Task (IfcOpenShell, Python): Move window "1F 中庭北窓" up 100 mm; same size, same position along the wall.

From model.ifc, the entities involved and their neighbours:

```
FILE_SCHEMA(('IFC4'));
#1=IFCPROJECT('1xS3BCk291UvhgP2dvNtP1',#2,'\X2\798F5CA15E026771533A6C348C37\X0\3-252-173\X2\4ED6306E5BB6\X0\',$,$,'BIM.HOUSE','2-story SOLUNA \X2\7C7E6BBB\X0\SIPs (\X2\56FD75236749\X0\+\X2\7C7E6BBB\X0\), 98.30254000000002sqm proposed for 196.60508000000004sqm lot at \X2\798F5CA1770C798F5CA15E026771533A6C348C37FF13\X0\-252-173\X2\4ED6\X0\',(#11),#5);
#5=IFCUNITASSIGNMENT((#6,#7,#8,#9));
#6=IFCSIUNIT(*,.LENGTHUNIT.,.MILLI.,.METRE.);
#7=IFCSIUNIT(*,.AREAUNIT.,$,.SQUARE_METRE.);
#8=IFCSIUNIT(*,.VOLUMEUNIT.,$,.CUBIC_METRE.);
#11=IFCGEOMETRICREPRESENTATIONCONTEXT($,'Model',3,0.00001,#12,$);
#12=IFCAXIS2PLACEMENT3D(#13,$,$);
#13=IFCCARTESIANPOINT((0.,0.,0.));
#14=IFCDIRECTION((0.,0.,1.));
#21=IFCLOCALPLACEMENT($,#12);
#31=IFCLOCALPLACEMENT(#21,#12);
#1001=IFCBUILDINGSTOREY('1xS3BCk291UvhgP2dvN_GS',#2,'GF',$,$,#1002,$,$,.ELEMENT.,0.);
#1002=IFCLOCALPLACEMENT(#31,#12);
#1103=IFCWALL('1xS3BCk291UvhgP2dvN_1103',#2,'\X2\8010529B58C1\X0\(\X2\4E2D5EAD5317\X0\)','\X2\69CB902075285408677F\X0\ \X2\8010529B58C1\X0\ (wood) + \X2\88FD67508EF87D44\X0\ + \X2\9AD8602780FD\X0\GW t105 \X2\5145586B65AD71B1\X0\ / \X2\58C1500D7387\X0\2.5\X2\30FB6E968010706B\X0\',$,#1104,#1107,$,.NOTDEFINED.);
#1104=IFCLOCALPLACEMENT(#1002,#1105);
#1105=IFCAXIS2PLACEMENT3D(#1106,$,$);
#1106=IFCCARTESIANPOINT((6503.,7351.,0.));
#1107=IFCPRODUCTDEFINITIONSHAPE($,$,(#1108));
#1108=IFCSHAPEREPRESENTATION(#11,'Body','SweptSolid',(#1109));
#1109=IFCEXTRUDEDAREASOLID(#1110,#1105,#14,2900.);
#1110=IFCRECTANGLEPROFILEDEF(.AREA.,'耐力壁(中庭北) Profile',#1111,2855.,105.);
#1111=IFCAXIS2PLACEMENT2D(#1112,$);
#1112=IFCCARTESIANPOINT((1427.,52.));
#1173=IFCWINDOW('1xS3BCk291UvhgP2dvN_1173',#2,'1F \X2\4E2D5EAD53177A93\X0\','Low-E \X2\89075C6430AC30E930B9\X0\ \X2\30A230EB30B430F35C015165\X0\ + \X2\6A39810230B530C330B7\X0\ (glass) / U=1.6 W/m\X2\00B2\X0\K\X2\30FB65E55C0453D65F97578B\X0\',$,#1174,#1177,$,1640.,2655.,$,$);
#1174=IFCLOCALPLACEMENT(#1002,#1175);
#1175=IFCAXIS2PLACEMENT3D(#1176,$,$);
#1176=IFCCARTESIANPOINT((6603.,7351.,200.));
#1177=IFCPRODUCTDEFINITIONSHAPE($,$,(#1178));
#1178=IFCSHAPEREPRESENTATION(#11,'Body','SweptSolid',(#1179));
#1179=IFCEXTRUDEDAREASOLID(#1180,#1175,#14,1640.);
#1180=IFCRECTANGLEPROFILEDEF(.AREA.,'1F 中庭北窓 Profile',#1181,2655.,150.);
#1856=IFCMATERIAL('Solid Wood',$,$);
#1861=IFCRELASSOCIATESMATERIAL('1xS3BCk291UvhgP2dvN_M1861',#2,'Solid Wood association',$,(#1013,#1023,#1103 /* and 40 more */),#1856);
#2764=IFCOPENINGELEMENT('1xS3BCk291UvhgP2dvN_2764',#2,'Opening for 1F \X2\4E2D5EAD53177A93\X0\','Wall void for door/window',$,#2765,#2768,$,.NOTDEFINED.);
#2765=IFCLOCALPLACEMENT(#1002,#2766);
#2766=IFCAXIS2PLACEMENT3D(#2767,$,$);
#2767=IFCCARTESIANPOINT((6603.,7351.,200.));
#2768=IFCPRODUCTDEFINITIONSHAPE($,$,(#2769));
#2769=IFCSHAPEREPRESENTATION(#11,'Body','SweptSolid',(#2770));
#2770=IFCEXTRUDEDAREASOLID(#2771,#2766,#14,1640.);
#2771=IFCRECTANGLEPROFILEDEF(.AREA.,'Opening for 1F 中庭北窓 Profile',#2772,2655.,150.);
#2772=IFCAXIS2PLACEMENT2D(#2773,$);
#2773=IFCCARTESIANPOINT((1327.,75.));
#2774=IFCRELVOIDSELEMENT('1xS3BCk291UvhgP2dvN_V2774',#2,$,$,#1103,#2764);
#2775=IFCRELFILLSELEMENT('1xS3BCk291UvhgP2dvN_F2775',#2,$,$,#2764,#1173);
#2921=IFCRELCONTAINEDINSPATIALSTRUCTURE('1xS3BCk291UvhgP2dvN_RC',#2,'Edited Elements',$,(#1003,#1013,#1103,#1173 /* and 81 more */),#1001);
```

```python
import numpy as np
import ifcopenshell
import ifcopenshell.api.geometry
import ifcopenshell.util.placement
import ifcopenshell.util.unit

model = ifcopenshell.open("model.ifc")
unit_scale = ifcopenshell.util.unit.calculate_unit_scale(model)

window = model.by_guid("1xS3BCk291UvhgP2dvN_1173")
opening = window.FillsVoids[0].RelatingOpeningElement
dz = 0.1 / unit_scale

shift = np.array([0.0, 0.0, dz])
# The window is not placed relative to its opening, so move both.
for product in (opening, window):
    matrix = ifcopenshell.util.placement.get_local_placement(product.ObjectPlacement)
    matrix[:3, 3] += shift
    ifcopenshell.api.geometry.edit_object_placement(model, product=product, matrix=matrix, is_si=False)

print(f"moved by {dz * unit_scale:+.3f} m")

model.write("model_edited.ifc")
```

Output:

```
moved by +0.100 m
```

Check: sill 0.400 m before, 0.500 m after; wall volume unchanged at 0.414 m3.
